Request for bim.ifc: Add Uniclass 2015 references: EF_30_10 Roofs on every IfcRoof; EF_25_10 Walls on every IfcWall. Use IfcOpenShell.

First a look at what the model holds.

```python
import ifcopenshell

model = ifcopenshell.open("bim.ifc")
print(model.schema)
print("classifications:", [c.Name for c in model.by_type("IfcClassification")])
for ifc_class in ("IfcDoor", "IfcRoof", "IfcStair", "IfcWall", "IfcWindow"):
    print(ifc_class, len(model.by_type(ifc_class)))
```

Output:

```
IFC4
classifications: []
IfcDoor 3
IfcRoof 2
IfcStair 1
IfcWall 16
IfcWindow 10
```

```python
import ifcopenshell
import ifcopenshell.api.classification

model = ifcopenshell.open("bim.ifc")

system = ifcopenshell.api.classification.add_classification(model, classification="Uniclass 2015")

codes = {
    "IfcRoof": ("EF_30_10", "Roofs"),
    "IfcWall": ("EF_25_10", "Walls"),
}
for ifc_class, (code, name) in codes.items():
    products = model.by_type(ifc_class)
    ifcopenshell.api.classification.add_reference(
        model, products=products, classification=system, identification=code, name=name
    )
    print(code, len(products))

model.write("bim_updated.ifc")
```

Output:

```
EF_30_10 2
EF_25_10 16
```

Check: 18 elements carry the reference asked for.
